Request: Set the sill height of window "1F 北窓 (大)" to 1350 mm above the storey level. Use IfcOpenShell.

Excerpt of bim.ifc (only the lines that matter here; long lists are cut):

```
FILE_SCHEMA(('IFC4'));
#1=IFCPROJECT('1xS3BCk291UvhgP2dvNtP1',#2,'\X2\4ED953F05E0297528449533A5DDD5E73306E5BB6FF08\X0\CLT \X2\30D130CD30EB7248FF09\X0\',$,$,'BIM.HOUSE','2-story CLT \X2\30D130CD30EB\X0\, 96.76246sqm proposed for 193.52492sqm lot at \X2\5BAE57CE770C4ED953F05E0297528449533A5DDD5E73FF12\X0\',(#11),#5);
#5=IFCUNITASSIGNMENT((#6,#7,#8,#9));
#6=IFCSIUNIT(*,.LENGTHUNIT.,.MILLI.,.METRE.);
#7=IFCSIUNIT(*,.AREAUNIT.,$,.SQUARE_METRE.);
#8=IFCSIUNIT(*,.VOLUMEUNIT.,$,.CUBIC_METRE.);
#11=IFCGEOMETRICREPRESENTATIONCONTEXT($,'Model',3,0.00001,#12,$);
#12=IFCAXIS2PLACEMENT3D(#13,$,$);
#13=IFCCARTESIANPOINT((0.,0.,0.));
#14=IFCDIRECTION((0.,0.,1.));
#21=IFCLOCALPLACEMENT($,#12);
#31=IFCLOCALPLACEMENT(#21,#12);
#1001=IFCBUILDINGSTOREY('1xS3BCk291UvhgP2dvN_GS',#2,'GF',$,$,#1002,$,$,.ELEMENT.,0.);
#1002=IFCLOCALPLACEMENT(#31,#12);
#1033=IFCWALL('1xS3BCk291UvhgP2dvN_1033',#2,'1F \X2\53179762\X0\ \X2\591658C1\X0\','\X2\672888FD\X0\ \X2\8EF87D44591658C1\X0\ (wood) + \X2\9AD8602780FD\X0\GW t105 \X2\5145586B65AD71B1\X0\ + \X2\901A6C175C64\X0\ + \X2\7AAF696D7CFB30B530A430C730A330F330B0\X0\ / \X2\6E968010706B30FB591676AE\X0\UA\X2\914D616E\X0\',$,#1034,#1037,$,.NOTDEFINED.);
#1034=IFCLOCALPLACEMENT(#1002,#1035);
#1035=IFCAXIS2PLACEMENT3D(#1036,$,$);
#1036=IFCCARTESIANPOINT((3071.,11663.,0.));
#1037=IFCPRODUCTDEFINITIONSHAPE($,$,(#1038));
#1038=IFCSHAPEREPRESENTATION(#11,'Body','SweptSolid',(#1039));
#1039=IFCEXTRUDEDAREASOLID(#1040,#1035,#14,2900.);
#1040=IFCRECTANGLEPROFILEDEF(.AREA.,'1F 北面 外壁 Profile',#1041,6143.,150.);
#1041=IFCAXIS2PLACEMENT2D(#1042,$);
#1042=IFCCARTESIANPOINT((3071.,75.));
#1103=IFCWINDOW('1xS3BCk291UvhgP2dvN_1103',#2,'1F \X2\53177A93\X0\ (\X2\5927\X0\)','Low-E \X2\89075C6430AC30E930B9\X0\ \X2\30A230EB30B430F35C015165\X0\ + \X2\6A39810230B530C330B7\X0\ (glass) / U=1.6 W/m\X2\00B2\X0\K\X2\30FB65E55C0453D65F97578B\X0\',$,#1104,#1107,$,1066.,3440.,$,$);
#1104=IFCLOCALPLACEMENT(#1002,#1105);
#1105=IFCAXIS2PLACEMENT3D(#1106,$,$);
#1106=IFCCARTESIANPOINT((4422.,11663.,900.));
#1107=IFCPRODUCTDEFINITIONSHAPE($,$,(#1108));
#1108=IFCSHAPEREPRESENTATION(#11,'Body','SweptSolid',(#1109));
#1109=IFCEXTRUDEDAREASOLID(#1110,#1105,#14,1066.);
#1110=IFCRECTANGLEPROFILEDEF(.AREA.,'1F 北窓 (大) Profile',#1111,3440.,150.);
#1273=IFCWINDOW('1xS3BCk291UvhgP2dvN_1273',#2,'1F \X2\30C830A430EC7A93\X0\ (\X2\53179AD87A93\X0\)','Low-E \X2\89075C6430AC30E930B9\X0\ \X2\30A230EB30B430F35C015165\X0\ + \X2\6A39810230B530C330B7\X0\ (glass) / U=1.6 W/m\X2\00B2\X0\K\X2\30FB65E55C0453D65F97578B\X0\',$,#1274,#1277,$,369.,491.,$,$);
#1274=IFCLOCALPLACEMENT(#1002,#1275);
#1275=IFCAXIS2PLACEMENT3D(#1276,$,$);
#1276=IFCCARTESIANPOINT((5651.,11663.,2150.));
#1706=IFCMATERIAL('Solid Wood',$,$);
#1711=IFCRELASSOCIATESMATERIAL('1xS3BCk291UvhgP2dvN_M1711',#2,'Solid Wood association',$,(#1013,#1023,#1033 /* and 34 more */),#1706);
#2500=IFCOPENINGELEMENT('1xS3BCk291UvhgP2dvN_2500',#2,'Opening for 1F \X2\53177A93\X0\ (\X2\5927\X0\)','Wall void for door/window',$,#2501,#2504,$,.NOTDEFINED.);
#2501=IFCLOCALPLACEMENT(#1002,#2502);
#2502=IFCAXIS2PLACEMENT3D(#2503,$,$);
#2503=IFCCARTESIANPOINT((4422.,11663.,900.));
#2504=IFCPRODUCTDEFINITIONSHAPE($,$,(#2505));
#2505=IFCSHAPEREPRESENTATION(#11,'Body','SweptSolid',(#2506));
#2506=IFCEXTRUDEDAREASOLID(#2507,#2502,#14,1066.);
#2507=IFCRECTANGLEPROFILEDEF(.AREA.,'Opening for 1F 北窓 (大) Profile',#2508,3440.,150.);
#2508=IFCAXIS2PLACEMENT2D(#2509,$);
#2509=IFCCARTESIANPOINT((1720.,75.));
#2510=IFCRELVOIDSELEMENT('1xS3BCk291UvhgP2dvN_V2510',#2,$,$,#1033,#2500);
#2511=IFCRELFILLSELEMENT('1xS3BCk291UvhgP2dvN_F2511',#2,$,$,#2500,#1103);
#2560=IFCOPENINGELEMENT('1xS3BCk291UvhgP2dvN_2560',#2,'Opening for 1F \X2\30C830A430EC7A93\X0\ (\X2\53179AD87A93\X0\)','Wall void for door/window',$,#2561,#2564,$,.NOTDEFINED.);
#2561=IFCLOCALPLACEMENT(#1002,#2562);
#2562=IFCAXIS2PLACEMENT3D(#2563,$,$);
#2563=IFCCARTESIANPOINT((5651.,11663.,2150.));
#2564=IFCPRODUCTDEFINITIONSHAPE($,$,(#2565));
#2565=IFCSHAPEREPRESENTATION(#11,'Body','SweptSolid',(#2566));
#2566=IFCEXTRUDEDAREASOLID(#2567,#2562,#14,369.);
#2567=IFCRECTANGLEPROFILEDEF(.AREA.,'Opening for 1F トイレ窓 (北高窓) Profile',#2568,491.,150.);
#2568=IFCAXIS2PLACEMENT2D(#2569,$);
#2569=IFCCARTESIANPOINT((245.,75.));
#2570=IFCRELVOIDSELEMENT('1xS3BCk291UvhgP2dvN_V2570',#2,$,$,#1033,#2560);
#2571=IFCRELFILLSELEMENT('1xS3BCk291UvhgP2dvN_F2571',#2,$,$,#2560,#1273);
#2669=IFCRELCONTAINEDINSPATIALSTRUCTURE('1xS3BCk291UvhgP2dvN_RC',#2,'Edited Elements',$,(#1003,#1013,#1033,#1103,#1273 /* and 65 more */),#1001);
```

```python
import numpy as np
import ifcopenshell
import ifcopenshell.api.geometry
import ifcopenshell.geom
import ifcopenshell.util.element
import ifcopenshell.util.placement
import ifcopenshell.util.shape
import ifcopenshell.util.unit

model = ifcopenshell.open("bim.ifc")
unit_scale = ifcopenshell.util.unit.calculate_unit_scale(model)

window = model.by_guid("1xS3BCk291UvhgP2dvN_1103")
opening = window.FillsVoids[0].RelatingOpeningElement
storey = ifcopenshell.util.element.get_container(window, ifc_class="IfcBuildingStorey")
level = ifcopenshell.util.placement.get_local_placement(storey.ObjectPlacement)[2, 3]

# The opening's origin need not be at the sill, so measure its lowest point.
shape = ifcopenshell.geom.create_shape(ifcopenshell.geom.settings(), opening)
bottom = ifcopenshell.util.shape.get_shape_bottom_elevation(shape, shape.geometry) / unit_scale
dz = level + 1.35 / unit_scale - bottom

shift = np.array([0.0, 0.0, dz])
# The window is not placed relative to its opening, so move both.
for product in (opening, window):
    matrix = ifcopenshell.util.placement.get_local_placement(product.ObjectPlacement)
    matrix[:3, 3] += shift
    ifcopenshell.api.geometry.edit_object_placement(model, product=product, matrix=matrix, is_si=False)

print(f"moved by {dz * unit_scale:+.3f} m")

model.write("bim_rev.ifc")
```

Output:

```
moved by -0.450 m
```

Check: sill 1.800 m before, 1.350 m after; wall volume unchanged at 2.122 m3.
